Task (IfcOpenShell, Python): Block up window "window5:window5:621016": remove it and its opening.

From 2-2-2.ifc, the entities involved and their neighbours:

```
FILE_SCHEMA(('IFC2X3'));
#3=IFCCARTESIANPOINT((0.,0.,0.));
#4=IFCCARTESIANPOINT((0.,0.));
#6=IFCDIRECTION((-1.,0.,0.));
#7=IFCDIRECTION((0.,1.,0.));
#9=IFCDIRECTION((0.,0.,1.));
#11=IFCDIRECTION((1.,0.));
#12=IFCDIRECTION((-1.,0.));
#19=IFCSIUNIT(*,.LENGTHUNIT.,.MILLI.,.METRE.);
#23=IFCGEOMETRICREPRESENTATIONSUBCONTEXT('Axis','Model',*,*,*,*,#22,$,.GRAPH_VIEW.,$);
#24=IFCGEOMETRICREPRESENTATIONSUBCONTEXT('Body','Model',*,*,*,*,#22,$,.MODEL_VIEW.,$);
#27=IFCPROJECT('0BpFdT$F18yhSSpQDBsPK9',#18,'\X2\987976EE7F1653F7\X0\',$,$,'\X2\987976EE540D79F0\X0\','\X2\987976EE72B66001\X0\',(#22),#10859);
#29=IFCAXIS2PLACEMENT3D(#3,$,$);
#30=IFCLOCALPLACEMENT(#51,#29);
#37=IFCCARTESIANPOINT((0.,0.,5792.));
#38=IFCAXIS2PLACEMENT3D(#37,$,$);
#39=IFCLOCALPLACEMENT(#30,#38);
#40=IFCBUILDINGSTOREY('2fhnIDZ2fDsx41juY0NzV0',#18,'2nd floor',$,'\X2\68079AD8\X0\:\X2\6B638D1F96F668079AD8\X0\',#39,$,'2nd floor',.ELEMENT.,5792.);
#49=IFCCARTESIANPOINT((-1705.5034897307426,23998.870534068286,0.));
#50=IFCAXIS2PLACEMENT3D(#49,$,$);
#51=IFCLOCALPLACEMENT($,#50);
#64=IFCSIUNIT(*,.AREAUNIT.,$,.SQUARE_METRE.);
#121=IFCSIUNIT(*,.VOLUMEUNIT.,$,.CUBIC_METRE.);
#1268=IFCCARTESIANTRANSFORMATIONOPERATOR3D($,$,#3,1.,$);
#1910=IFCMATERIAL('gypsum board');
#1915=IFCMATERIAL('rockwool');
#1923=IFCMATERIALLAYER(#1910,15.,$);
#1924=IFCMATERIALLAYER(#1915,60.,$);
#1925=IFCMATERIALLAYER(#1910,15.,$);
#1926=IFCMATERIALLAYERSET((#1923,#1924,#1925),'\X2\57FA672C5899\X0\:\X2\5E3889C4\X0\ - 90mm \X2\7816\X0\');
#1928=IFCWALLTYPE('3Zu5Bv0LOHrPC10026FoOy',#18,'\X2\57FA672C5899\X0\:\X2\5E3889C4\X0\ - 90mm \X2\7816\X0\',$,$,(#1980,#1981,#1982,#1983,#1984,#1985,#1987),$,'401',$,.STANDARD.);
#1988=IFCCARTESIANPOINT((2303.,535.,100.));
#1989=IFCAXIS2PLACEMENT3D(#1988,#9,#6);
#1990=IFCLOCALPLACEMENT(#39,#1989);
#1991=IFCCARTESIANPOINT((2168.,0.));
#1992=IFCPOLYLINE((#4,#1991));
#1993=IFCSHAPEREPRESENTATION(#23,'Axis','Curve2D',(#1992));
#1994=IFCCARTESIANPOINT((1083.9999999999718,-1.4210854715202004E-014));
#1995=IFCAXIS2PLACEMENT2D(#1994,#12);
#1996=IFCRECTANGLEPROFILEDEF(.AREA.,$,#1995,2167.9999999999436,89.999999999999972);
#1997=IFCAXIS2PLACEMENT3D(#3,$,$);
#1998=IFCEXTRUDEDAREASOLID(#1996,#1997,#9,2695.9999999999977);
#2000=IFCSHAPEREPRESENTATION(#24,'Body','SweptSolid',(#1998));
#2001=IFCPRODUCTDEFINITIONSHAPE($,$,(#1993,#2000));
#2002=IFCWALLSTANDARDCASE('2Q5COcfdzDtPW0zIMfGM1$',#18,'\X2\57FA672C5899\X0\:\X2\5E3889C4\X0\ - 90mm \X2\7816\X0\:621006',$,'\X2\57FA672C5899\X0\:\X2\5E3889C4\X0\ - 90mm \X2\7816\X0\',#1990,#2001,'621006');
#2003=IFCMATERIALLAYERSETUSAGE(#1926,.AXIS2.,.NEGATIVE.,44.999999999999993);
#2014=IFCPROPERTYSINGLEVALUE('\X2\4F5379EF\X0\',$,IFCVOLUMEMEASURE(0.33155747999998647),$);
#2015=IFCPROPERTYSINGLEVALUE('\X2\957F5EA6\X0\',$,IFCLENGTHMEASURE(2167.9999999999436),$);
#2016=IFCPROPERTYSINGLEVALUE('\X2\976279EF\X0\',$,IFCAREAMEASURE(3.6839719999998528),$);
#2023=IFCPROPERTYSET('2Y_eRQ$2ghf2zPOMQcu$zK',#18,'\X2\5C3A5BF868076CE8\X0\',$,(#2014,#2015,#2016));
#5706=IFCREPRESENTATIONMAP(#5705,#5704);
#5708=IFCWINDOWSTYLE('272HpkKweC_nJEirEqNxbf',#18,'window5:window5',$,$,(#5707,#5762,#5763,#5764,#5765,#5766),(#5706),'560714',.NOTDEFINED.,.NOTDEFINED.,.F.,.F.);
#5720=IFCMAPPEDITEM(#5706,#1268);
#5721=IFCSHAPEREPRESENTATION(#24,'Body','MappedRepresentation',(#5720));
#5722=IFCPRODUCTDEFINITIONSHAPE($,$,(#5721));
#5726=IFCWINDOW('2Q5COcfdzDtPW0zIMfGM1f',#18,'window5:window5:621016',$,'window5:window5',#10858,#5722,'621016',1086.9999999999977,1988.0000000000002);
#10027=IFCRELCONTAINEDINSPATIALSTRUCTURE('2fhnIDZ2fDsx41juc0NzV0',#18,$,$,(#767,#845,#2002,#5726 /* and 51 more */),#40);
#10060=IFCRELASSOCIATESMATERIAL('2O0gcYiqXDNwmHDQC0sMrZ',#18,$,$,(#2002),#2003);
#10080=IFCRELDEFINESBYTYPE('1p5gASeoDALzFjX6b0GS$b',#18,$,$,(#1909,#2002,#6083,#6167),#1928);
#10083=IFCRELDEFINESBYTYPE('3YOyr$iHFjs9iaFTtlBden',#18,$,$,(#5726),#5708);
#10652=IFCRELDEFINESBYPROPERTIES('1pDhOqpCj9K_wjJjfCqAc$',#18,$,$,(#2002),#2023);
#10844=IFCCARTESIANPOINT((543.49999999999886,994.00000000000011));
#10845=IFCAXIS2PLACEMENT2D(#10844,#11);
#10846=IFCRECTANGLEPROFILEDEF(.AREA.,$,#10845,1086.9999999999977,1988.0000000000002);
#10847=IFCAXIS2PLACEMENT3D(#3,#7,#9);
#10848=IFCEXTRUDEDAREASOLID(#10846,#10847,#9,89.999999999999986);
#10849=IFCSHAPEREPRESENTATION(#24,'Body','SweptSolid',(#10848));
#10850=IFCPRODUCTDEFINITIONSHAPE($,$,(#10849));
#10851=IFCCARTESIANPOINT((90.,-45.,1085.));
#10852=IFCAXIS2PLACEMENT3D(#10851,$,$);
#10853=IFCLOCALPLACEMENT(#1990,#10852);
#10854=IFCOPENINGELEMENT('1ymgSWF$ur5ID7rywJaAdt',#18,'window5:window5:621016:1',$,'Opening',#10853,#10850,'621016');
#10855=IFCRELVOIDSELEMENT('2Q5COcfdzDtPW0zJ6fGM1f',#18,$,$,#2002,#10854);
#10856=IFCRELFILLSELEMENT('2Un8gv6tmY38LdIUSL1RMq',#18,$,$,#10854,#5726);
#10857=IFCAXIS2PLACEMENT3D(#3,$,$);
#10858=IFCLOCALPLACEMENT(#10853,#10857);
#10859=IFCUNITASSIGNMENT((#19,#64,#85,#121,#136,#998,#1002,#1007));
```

```python
import ifcopenshell
import ifcopenshell.api.feature
import ifcopenshell.api.pset
import ifcopenshell.api.root
import ifcopenshell.geom
import ifcopenshell.util.element
import ifcopenshell.util.shape
import ifcopenshell.util.unit

model = ifcopenshell.open("2-2-2.ifc")
area_scale = ifcopenshell.util.unit.calculate_unit_scale(model, "AREAUNIT")
volume_scale = ifcopenshell.util.unit.calculate_unit_scale(model, "VOLUMEUNIT")
settings = ifcopenshell.geom.settings()


def volume(element):
    """Net volume in cubic metres, openings subtracted."""
    shape = ifcopenshell.geom.create_shape(settings, element)
    return ifcopenshell.util.shape.get_volume(shape.geometry)


window = model.by_guid("2Q5COcfdzDtPW0zIMfGM1f")
opening = window.FillsVoids[0].RelatingOpeningElement
wall = opening.VoidsElements[0].RelatingBuildingElement
before = volume(wall)

ifcopenshell.api.root.remove_product(model, product=window)
ifcopenshell.api.feature.remove_feature(model, feature=opening)

after = volume(wall)
thickness = 0.09  # wall thickness in metres

# Update the wall's stored quantities.
pset = model.by_id(ifcopenshell.util.element.get_pset(wall, "尺寸标注", should_inherit=False)["id"])
ifcopenshell.api.pset.edit_pset(model, pset=pset, properties={
    "体积": model.create_entity("IfcVolumeMeasure", after / volume_scale),
    "面积": model.create_entity("IfcAreaMeasure", after / thickness / area_scale),
})

print(f"wall volume {before:.3f} -> {after:.3f} m3")

model.write("2-2-2_updated.ifc")
```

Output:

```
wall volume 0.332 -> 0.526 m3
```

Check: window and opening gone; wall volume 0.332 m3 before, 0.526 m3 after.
